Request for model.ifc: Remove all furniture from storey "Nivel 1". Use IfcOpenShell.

First a look at what the model holds.

```python
import ifcopenshell
import ifcopenshell.util.element

model = ifcopenshell.open("model.ifc")
print(model.schema)
storey = next(s for s in model.by_type("IfcBuildingStorey") if s.Name == "Nivel 1")
furniture = [e for e in ifcopenshell.util.element.get_decomposition(storey) if e.is_a("IfcFurnishingElement")]
seen = {}
for e in furniture:
    element_type = ifcopenshell.util.element.get_type(e)
    name = element_type.Name if element_type not in (None, e) else None
    seen[name] = seen.get(name, 0) + 1
for name, count in sorted(seen.items(), key=str):
    print(count, "x", name)
```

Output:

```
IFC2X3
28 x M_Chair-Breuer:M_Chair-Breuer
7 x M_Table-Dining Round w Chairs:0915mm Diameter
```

```python
import ifcopenshell
import ifcopenshell.api.root
import ifcopenshell.util.element

model = ifcopenshell.open("model.ifc")

storey = next(s for s in model.by_type("IfcBuildingStorey") if s.Name == "Nivel 1")
furniture = [e for e in ifcopenshell.util.element.get_decomposition(storey) if e.is_a("IfcFurnishingElement")]

for e in furniture:
    ifcopenshell.api.root.remove_product(model, product=e)
print(len(furniture), "removed")

model.write("model-out.ifc")
```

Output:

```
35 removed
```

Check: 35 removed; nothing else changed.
